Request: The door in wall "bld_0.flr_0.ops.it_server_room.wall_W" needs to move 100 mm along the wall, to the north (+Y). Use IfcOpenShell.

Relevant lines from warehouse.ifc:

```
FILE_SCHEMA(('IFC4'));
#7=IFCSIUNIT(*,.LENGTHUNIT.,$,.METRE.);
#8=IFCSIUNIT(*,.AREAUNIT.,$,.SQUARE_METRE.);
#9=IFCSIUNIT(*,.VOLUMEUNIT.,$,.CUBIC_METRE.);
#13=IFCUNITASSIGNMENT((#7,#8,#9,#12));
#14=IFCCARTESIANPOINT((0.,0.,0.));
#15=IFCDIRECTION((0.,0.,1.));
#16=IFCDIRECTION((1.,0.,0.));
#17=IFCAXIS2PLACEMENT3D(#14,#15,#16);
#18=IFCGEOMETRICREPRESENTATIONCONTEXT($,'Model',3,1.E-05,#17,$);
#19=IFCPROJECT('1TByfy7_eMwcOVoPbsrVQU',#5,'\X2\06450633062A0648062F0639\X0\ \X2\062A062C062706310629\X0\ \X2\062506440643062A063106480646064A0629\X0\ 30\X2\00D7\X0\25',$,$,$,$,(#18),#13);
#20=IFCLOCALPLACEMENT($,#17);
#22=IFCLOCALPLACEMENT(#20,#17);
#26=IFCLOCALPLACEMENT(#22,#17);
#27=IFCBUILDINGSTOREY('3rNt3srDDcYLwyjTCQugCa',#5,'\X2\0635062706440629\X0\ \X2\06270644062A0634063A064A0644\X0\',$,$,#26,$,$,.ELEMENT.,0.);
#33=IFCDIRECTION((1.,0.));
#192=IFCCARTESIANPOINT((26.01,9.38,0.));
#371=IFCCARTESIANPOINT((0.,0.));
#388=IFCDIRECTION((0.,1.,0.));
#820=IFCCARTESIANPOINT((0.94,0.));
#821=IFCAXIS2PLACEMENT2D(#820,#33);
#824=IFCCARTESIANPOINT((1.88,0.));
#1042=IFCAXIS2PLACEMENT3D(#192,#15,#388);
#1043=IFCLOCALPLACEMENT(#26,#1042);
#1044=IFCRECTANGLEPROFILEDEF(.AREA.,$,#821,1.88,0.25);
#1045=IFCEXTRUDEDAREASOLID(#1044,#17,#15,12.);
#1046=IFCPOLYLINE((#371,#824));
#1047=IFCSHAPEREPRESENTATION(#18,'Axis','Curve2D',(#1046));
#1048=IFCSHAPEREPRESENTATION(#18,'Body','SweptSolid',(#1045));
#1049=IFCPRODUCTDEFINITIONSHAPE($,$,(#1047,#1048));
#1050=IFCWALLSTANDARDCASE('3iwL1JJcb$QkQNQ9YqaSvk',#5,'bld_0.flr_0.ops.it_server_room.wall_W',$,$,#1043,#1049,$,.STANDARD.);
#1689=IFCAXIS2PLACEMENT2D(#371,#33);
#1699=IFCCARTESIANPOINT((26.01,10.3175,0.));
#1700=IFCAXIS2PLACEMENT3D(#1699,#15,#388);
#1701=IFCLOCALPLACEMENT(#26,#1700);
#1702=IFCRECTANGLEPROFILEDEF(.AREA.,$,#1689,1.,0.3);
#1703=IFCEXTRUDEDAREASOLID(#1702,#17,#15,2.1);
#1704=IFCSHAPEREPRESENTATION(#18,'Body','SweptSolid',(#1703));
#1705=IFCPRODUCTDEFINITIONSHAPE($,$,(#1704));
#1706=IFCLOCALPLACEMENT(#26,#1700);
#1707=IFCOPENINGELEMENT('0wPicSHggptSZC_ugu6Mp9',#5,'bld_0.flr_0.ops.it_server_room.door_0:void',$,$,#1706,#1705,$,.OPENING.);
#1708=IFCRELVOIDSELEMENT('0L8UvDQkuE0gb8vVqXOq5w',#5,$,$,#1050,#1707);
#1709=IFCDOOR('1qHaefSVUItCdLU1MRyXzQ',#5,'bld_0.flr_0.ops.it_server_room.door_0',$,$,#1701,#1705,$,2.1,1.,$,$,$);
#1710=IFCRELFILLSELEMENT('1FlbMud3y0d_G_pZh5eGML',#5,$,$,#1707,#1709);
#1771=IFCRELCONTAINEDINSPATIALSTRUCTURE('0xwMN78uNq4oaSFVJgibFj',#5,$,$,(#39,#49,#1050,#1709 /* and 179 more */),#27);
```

```python
import ifcopenshell
import ifcopenshell.api.geometry
import ifcopenshell.util.placement
import ifcopenshell.util.unit

model = ifcopenshell.open("warehouse.ifc")
unit_scale = ifcopenshell.util.unit.calculate_unit_scale(model)

door = model.by_guid("1qHaefSVUItCdLU1MRyXzQ")
opening = door.FillsVoids[0].RelatingOpeningElement
wall = opening.VoidsElements[0].RelatingBuildingElement

wall_matrix = ifcopenshell.util.placement.get_local_placement(wall.ObjectPlacement)
shift = wall_matrix[:3, 0] * 0.1 / unit_scale
before = ifcopenshell.util.placement.get_local_placement(door.ObjectPlacement)[:3, 3].copy()

# The door is not placed relative to its opening, so move both.
for product in (opening, door):
    matrix = ifcopenshell.util.placement.get_local_placement(product.ObjectPlacement)
    matrix[:3, 3] += shift
    ifcopenshell.api.geometry.edit_object_placement(model, product=product, matrix=matrix, is_si=False)

after = ifcopenshell.util.placement.get_local_placement(door.ObjectPlacement)[:3, 3]
print("door moved by", (after - before).round(3) + 0.0)

model.write("warehouse_v2.ifc")
```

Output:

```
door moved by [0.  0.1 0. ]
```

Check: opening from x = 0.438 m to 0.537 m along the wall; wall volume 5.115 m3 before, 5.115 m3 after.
